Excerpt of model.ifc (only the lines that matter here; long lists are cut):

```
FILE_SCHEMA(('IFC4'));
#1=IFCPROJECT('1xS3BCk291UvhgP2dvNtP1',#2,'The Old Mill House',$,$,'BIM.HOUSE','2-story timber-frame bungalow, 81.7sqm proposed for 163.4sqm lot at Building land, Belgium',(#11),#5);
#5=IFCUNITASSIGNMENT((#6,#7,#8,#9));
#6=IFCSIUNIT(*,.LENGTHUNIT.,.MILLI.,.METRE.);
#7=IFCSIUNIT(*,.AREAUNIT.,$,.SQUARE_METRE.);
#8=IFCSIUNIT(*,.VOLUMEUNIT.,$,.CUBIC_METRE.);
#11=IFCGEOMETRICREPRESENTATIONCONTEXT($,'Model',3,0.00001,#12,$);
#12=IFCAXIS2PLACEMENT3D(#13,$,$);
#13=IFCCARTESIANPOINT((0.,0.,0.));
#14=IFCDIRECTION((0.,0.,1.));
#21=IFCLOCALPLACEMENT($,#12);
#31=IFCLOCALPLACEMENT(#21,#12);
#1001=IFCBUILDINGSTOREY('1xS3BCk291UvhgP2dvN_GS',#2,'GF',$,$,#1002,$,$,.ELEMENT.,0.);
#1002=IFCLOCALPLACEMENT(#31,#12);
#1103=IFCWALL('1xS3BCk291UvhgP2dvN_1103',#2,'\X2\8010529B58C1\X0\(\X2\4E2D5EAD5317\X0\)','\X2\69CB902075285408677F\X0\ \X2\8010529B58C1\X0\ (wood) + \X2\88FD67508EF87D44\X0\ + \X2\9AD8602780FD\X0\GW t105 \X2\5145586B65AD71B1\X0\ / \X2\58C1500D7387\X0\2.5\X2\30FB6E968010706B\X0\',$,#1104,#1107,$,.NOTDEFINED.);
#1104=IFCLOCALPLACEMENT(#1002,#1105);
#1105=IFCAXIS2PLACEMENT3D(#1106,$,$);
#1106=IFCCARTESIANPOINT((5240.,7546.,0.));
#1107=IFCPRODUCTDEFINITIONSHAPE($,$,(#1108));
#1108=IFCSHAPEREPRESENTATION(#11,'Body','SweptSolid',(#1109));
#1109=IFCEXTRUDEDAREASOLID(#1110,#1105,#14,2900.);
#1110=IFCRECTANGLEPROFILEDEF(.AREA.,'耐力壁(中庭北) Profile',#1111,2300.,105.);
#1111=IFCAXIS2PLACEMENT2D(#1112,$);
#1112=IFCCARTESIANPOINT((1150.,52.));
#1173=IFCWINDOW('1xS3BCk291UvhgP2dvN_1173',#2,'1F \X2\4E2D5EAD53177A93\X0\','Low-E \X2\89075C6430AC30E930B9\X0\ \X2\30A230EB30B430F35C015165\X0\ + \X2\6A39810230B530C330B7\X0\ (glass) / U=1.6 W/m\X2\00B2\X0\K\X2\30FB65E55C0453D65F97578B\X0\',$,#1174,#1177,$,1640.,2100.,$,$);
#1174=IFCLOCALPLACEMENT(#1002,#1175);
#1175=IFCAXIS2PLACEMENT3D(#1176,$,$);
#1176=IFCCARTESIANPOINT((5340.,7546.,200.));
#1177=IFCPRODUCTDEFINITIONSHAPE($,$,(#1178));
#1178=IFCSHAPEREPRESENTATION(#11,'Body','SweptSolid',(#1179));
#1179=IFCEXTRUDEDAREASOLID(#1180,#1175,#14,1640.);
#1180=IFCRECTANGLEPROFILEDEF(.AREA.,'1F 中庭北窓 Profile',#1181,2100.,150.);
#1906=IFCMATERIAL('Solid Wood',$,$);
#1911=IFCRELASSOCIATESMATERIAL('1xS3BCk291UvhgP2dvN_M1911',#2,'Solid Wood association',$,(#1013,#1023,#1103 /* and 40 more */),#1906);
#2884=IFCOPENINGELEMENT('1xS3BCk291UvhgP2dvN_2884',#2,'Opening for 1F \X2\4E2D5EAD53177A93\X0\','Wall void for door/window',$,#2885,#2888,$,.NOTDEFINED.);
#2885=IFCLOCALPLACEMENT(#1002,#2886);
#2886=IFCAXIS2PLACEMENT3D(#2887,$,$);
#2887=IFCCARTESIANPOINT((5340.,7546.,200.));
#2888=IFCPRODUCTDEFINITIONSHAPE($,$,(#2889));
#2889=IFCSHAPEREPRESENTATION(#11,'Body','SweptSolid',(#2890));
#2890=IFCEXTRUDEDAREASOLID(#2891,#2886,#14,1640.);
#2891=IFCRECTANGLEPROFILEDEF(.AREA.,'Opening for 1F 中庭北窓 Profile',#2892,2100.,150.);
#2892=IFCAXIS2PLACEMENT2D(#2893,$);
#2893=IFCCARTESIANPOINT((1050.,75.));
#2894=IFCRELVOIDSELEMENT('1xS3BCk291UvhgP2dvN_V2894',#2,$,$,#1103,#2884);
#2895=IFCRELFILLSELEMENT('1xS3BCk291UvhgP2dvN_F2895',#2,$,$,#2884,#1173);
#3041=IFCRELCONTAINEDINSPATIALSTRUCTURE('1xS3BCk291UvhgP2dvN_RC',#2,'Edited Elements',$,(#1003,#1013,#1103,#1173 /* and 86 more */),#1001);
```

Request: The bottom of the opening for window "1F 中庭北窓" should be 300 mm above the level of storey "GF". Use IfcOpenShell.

```python
import numpy as np
import ifcopenshell
import ifcopenshell.api.geometry
import ifcopenshell.geom
import ifcopenshell.util.element
import ifcopenshell.util.placement
import ifcopenshell.util.shape
import ifcopenshell.util.unit

model = ifcopenshell.open("model.ifc")
unit_scale = ifcopenshell.util.unit.calculate_unit_scale(model)

window = model.by_guid("1xS3BCk291UvhgP2dvN_1173")
opening = window.FillsVoids[0].RelatingOpeningElement
storey = ifcopenshell.util.element.get_container(window, ifc_class="IfcBuildingStorey")
level = ifcopenshell.util.placement.get_local_placement(storey.ObjectPlacement)[2, 3]

# The opening's origin need not be at the sill, so measure its lowest point.
shape = ifcopenshell.geom.create_shape(ifcopenshell.geom.settings(), opening)
bottom = ifcopenshell.util.shape.get_shape_bottom_elevation(shape, shape.geometry) / unit_scale
dz = level + 0.3 / unit_scale - bottom

shift = np.array([0.0, 0.0, dz])
# The window is not placed relative to its opening, so move both.
for product in (opening, window):
    matrix = ifcopenshell.util.placement.get_local_placement(product.ObjectPlacement)
    matrix[:3, 3] += shift
    ifcopenshell.api.geometry.edit_object_placement(model, product=product, matrix=matrix, is_si=False)

print(f"moved by {dz * unit_scale:+.3f} m")

model.write("model-out.ifc")
```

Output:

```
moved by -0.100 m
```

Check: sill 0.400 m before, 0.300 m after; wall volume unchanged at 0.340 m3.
